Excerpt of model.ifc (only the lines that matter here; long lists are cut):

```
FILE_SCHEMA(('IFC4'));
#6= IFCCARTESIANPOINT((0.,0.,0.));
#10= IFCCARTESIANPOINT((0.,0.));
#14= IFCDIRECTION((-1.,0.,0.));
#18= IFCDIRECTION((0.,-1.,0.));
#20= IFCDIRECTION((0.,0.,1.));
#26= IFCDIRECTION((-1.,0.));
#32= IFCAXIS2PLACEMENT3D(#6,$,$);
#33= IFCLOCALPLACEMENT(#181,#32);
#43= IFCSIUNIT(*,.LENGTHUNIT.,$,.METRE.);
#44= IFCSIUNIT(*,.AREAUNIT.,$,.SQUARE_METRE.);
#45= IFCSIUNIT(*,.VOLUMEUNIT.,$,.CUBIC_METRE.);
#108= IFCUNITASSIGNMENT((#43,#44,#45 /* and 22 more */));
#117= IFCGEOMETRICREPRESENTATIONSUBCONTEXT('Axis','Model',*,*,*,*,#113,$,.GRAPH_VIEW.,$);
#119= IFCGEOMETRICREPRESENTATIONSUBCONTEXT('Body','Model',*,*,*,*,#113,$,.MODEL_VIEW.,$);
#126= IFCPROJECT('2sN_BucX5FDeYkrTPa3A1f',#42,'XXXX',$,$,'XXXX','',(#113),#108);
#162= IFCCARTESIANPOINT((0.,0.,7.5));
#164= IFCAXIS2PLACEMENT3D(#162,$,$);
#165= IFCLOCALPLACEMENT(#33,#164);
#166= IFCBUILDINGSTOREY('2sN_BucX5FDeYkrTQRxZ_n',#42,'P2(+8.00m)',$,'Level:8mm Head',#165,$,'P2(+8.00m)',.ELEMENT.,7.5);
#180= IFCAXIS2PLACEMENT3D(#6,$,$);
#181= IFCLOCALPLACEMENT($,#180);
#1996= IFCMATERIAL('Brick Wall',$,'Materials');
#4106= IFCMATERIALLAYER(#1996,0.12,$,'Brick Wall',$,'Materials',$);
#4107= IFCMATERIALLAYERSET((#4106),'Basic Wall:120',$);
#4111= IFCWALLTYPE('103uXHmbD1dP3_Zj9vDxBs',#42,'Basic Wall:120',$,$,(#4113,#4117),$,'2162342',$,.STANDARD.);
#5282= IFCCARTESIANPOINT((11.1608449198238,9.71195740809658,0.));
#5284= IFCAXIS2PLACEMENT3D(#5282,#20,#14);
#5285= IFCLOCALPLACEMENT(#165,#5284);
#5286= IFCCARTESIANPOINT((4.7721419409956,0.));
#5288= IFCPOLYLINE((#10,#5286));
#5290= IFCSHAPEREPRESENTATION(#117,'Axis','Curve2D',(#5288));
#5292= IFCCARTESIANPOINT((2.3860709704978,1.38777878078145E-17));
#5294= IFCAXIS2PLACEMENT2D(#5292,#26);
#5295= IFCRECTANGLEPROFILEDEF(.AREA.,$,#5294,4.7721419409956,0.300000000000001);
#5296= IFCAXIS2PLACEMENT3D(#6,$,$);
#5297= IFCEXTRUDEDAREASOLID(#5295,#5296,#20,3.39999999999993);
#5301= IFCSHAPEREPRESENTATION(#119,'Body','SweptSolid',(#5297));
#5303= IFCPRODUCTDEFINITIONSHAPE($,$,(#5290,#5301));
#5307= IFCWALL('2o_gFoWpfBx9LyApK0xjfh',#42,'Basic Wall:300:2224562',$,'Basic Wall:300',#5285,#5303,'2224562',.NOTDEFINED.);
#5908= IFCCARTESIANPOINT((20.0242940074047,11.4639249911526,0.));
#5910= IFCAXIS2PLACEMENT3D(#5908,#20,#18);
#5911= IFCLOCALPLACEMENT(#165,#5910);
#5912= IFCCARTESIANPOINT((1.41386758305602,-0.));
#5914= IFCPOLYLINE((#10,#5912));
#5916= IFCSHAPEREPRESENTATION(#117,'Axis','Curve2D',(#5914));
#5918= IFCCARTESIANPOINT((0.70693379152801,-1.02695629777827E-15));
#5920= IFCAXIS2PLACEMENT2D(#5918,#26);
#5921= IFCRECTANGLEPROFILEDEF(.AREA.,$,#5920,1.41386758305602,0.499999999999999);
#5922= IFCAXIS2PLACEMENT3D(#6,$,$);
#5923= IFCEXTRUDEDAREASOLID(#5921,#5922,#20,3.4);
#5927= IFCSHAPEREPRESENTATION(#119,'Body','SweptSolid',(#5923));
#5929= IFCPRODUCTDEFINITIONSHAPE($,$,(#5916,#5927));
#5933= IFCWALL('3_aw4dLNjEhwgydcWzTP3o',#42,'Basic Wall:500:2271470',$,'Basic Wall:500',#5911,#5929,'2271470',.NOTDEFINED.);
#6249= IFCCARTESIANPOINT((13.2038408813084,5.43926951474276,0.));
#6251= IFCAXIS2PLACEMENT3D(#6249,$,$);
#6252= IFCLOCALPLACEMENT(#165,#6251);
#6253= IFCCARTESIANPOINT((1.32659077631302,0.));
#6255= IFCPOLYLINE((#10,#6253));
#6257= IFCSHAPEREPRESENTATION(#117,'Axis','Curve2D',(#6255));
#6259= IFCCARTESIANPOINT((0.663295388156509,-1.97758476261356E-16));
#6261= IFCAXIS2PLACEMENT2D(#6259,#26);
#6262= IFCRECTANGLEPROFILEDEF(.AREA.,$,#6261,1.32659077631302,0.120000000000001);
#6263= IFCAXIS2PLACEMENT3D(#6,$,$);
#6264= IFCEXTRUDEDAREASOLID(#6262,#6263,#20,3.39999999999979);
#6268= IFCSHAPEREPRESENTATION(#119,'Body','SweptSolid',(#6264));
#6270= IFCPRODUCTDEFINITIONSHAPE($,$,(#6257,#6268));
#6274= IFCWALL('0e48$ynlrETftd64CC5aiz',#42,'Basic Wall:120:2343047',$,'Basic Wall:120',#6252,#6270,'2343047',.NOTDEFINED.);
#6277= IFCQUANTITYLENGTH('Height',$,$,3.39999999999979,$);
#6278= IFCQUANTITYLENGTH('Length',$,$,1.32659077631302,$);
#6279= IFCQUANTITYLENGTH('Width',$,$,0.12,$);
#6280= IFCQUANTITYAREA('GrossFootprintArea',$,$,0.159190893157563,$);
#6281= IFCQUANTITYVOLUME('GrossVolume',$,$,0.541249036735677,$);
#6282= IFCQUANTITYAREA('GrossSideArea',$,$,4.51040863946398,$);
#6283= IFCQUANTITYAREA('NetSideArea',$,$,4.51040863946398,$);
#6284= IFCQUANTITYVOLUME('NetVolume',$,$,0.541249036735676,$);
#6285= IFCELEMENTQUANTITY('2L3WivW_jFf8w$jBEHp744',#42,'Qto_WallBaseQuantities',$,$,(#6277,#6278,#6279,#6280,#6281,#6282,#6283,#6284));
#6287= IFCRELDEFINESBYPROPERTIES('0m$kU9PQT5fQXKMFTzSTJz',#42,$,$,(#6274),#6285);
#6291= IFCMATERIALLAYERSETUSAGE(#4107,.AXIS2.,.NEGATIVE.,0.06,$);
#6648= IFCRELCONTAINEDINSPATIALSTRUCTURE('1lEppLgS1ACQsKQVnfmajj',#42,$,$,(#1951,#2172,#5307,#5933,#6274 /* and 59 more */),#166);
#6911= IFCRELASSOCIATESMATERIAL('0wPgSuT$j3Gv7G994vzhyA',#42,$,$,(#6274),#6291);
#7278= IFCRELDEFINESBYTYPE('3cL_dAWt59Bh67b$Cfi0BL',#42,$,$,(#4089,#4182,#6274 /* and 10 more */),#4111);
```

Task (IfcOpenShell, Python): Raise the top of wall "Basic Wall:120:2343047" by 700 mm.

```python
import ifcopenshell
import ifcopenshell.api.pset
import ifcopenshell.geom
import ifcopenshell.util.element
import ifcopenshell.util.representation
import ifcopenshell.util.shape
import ifcopenshell.util.unit

model = ifcopenshell.open("model.ifc")
unit_scale = ifcopenshell.util.unit.calculate_unit_scale(model)
area_scale = ifcopenshell.util.unit.calculate_unit_scale(model, "AREAUNIT")
volume_scale = ifcopenshell.util.unit.calculate_unit_scale(model, "VOLUMEUNIT")
settings = ifcopenshell.geom.settings()


def volume(element):
    """Net volume in cubic metres, openings subtracted."""
    shape = ifcopenshell.geom.create_shape(settings, element)
    return ifcopenshell.util.shape.get_volume(shape.geometry)


wall = model.by_guid("0e48$ynlrETftd64CC5aiz")
before = volume(wall)

body = ifcopenshell.util.representation.get_representation(wall, "Model", "Body")
solid = body.Items[0]
old_height = solid.Depth
solid.Depth += 0.7 / unit_scale
after = volume(wall)
thickness = 0.12  # wall thickness in metres

# Update the stored height, areas and volumes.
qto = model.by_id(ifcopenshell.util.element.get_pset(wall, "Qto_WallBaseQuantities", should_inherit=False)["id"])
ifcopenshell.api.pset.edit_qto(model, qto=qto, properties={
    "Height": solid.Depth,
    "GrossVolume": ifcopenshell.util.element.get_pset(wall, "Qto_WallBaseQuantities", "GrossVolume") * solid.Depth / old_height,
    "GrossSideArea": ifcopenshell.util.element.get_pset(wall, "Qto_WallBaseQuantities", "GrossSideArea") * solid.Depth / old_height,
    "NetSideArea": after / thickness / area_scale,
    "NetVolume": after / volume_scale,
})

print(f"height {old_height:g} -> {solid.Depth:g}, volume {before:.3f} -> {after:.3f} m3")

model.write("model_v2.ifc")
```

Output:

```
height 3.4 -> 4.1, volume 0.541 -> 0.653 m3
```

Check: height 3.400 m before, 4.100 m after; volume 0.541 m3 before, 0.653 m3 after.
